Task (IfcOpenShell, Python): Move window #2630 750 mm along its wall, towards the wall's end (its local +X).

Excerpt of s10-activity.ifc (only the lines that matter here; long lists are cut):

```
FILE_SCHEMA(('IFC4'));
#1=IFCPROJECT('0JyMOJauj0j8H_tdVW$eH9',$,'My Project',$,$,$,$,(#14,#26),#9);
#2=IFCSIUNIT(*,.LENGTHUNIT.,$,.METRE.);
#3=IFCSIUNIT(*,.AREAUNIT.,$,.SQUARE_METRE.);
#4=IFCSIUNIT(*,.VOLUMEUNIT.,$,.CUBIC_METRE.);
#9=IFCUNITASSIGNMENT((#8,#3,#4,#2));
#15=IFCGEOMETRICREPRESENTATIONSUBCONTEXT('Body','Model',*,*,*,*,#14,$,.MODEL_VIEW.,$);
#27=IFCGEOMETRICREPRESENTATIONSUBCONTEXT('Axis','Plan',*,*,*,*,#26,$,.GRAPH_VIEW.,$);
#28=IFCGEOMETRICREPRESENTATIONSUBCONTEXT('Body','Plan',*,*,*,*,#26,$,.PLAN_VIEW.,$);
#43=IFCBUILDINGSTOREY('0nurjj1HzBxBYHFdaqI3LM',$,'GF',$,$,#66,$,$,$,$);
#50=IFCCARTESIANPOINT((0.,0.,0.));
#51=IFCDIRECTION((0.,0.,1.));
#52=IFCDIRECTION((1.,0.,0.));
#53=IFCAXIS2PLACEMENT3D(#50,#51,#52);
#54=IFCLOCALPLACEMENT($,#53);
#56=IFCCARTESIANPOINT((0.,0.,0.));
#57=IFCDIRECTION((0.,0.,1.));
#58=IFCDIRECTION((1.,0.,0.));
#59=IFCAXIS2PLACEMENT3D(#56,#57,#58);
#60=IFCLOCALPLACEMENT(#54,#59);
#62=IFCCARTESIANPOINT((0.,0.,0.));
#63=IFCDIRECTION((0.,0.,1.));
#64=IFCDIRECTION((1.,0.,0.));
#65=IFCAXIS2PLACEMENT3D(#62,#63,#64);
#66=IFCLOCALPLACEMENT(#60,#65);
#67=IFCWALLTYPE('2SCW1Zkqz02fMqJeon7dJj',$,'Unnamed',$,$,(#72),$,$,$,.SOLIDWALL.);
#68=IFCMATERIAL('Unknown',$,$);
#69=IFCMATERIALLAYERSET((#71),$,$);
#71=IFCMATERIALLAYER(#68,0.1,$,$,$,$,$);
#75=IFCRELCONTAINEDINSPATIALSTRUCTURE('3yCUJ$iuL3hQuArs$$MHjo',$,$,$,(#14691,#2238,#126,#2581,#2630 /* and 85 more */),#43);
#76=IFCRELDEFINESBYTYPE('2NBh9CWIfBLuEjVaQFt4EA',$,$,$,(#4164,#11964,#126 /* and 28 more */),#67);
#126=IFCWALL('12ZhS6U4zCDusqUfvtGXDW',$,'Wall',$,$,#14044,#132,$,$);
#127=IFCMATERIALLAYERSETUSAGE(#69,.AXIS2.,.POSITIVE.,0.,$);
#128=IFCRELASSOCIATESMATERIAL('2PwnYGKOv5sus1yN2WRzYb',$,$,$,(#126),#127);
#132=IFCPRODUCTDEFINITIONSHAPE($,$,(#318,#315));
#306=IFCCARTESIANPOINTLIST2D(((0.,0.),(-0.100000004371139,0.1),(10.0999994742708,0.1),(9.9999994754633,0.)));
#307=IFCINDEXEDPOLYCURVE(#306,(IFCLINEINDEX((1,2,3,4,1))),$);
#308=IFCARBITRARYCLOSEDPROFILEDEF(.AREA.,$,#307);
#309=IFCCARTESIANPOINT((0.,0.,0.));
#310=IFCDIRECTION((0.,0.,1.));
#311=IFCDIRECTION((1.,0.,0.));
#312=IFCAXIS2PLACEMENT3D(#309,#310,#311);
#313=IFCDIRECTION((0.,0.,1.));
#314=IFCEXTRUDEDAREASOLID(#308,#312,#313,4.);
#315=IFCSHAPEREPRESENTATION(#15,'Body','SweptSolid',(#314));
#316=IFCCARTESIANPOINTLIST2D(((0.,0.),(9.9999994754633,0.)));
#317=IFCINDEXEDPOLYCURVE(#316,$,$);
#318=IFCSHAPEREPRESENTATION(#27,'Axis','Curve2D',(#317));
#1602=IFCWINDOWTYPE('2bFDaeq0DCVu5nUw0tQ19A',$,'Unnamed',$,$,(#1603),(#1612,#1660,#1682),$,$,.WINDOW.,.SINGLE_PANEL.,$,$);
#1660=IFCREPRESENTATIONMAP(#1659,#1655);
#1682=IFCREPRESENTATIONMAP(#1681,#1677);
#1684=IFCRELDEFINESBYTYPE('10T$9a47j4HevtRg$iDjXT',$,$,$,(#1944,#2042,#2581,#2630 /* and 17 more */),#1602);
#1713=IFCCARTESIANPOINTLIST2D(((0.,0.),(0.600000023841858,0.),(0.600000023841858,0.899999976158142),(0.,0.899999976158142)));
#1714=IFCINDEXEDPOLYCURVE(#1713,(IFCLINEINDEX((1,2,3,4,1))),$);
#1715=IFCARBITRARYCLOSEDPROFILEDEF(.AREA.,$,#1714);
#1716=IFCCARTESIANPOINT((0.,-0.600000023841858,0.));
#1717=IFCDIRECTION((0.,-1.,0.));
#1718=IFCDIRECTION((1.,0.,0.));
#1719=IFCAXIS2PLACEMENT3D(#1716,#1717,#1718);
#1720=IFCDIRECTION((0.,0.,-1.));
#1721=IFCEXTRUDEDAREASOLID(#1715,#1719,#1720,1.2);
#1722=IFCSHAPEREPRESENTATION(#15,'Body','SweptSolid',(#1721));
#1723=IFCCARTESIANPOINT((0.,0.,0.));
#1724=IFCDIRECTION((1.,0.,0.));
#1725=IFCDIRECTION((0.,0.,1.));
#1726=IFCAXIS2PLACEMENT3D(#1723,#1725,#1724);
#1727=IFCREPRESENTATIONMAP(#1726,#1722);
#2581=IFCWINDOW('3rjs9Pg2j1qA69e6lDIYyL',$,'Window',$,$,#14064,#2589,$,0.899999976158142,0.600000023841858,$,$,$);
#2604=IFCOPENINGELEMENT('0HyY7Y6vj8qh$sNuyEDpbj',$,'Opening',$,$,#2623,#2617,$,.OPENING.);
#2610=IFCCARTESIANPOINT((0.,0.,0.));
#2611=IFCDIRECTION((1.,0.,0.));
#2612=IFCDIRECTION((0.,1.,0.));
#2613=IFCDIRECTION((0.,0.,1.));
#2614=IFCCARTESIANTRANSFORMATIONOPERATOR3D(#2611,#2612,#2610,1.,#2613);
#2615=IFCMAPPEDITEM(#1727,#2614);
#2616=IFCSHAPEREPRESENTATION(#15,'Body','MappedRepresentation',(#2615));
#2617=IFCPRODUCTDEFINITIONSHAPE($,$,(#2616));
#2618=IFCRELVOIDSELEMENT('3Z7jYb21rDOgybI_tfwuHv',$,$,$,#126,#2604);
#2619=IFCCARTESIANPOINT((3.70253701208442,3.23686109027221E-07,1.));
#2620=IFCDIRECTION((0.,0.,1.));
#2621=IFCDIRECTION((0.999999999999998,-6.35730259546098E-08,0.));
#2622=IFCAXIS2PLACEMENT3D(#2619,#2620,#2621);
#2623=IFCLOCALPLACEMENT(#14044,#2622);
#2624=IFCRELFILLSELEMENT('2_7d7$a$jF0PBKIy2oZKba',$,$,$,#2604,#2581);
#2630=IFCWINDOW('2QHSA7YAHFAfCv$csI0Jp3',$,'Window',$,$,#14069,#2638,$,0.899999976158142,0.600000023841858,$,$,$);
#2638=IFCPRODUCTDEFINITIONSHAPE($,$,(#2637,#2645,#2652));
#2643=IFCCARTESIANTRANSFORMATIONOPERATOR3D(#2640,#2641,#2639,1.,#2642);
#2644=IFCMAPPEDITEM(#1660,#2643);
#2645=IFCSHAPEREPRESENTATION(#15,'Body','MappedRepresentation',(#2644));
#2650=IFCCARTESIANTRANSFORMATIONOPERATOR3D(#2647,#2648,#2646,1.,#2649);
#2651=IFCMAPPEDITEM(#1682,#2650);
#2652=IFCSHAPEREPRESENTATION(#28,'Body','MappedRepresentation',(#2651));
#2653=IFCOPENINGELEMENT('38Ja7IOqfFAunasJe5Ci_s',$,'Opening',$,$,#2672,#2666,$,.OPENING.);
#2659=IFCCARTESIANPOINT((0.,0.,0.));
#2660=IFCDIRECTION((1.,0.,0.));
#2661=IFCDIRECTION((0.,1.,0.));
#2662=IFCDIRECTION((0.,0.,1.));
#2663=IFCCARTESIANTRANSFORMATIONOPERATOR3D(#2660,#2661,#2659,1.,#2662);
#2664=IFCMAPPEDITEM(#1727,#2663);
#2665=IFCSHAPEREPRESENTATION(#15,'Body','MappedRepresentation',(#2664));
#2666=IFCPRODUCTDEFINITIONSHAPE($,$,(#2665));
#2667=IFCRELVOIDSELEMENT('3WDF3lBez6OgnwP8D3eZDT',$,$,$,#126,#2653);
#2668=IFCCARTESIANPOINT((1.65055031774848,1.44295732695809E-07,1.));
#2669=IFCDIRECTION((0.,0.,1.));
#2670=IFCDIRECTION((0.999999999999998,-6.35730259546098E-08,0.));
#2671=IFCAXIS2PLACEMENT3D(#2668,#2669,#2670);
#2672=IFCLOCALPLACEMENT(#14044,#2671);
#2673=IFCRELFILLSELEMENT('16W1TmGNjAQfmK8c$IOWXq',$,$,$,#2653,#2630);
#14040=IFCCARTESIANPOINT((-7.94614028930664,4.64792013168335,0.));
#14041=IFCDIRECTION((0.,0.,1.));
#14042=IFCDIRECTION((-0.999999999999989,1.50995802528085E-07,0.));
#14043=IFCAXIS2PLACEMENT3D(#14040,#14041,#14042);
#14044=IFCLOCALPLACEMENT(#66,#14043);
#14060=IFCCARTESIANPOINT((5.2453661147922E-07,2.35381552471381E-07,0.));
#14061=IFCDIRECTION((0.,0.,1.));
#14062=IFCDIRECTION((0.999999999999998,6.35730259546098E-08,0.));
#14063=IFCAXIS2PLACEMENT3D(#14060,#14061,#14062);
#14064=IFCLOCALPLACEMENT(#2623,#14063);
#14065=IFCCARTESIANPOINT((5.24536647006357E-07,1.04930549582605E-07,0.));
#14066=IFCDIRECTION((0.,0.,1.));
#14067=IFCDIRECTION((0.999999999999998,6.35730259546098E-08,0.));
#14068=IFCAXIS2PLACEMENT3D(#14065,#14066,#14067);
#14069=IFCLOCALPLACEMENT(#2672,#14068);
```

```python
import ifcopenshell
import ifcopenshell.api.geometry
import ifcopenshell.util.placement
import ifcopenshell.util.unit

model = ifcopenshell.open("s10-activity.ifc")
unit_scale = ifcopenshell.util.unit.calculate_unit_scale(model)

window = model.by_id(2630)
opening = window.FillsVoids[0].RelatingOpeningElement
wall = opening.VoidsElements[0].RelatingBuildingElement

wall_matrix = ifcopenshell.util.placement.get_local_placement(wall.ObjectPlacement)
shift = wall_matrix[:3, 0] * 0.75 / unit_scale
before = ifcopenshell.util.placement.get_local_placement(window.ObjectPlacement)[:3, 3].copy()

# The window is placed relative to its opening, so it follows when the opening moves.
matrix = ifcopenshell.util.placement.get_local_placement(opening.ObjectPlacement)
matrix[:3, 3] += shift
ifcopenshell.api.geometry.edit_object_placement(
    model, product=opening, matrix=matrix, is_si=False, should_transform_children=True
)

after = ifcopenshell.util.placement.get_local_placement(window.ObjectPlacement)[:3, 3]
print("window moved by", (after - before).round(3) + 0.0)

model.write("s10-activity_updated.ifc")
```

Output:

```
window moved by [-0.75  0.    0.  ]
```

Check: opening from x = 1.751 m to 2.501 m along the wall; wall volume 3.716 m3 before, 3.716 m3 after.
